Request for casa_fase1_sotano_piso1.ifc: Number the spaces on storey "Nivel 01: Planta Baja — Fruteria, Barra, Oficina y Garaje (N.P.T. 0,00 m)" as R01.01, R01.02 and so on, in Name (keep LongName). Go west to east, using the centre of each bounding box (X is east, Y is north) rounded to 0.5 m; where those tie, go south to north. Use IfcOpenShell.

First a look at what the model holds.

```python
import ifcopenshell
import ifcopenshell.util.element
import ifcopenshell.util.placement

model = ifcopenshell.open("casa_fase1_sotano_piso1.ifc")
print(model.schema)
storey = next(s for s in model.by_type("IfcBuildingStorey") if s.Name == "Nivel 01: Planta Baja — Fruteria, Barra, Oficina y Garaje (N.P.T. 0,00 m)")
spaces = [e for e in ifcopenshell.util.element.get_decomposition(storey) if e.is_a("IfcSpace")]
for e in sorted(spaces, key=lambda e: e.id()):
    origin = ifcopenshell.util.placement.get_local_placement(e.ObjectPlacement)[:3, 3]
    print(e.id(), e.Name, e.LongName, origin.round(2) + 0.0, sep=" | ")
```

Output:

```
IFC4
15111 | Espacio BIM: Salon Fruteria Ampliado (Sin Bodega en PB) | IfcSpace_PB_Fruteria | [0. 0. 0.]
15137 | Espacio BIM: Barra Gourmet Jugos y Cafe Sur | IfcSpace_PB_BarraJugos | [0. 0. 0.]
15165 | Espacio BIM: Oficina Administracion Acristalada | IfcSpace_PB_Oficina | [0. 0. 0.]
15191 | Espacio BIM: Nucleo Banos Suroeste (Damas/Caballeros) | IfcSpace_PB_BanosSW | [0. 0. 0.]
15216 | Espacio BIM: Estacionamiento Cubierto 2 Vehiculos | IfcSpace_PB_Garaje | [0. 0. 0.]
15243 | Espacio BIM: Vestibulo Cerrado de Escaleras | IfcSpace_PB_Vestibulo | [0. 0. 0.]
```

```python
import ifcopenshell
import ifcopenshell.geom
import ifcopenshell.util.element
import ifcopenshell.util.shape

model = ifcopenshell.open("casa_fase1_sotano_piso1.ifc")
settings = ifcopenshell.geom.settings()
settings.set("use-world-coords", True)


def centre(element):
    shape = ifcopenshell.geom.create_shape(settings, element)
    return ifcopenshell.util.shape.get_bbox_centroid(shape.geometry)


storey = next(s for s in model.by_type("IfcBuildingStorey") if s.Name == "Nivel 01: Planta Baja — Fruteria, Barra, Oficina y Garaje (N.P.T. 0,00 m)")
spaces = [e for e in ifcopenshell.util.element.get_decomposition(storey) if e.is_a("IfcSpace")]

# Insertion points can sit at a corner or the storey origin, so sort by the geometry (in metres).
centres = {e: centre(e) for e in spaces}
spaces.sort(key=lambda e: (round(centres[e][0] / 0.5), centres[e][1]))

for i, e in enumerate(spaces, start=1):
    number = f"R01.{i:02d}"
    e.Name = number
    print(e.id(), number)

model.write("casa_fase1_sotano_piso1_updated.ifc")
```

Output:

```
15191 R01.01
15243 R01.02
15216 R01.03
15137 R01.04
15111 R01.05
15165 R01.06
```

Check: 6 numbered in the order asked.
